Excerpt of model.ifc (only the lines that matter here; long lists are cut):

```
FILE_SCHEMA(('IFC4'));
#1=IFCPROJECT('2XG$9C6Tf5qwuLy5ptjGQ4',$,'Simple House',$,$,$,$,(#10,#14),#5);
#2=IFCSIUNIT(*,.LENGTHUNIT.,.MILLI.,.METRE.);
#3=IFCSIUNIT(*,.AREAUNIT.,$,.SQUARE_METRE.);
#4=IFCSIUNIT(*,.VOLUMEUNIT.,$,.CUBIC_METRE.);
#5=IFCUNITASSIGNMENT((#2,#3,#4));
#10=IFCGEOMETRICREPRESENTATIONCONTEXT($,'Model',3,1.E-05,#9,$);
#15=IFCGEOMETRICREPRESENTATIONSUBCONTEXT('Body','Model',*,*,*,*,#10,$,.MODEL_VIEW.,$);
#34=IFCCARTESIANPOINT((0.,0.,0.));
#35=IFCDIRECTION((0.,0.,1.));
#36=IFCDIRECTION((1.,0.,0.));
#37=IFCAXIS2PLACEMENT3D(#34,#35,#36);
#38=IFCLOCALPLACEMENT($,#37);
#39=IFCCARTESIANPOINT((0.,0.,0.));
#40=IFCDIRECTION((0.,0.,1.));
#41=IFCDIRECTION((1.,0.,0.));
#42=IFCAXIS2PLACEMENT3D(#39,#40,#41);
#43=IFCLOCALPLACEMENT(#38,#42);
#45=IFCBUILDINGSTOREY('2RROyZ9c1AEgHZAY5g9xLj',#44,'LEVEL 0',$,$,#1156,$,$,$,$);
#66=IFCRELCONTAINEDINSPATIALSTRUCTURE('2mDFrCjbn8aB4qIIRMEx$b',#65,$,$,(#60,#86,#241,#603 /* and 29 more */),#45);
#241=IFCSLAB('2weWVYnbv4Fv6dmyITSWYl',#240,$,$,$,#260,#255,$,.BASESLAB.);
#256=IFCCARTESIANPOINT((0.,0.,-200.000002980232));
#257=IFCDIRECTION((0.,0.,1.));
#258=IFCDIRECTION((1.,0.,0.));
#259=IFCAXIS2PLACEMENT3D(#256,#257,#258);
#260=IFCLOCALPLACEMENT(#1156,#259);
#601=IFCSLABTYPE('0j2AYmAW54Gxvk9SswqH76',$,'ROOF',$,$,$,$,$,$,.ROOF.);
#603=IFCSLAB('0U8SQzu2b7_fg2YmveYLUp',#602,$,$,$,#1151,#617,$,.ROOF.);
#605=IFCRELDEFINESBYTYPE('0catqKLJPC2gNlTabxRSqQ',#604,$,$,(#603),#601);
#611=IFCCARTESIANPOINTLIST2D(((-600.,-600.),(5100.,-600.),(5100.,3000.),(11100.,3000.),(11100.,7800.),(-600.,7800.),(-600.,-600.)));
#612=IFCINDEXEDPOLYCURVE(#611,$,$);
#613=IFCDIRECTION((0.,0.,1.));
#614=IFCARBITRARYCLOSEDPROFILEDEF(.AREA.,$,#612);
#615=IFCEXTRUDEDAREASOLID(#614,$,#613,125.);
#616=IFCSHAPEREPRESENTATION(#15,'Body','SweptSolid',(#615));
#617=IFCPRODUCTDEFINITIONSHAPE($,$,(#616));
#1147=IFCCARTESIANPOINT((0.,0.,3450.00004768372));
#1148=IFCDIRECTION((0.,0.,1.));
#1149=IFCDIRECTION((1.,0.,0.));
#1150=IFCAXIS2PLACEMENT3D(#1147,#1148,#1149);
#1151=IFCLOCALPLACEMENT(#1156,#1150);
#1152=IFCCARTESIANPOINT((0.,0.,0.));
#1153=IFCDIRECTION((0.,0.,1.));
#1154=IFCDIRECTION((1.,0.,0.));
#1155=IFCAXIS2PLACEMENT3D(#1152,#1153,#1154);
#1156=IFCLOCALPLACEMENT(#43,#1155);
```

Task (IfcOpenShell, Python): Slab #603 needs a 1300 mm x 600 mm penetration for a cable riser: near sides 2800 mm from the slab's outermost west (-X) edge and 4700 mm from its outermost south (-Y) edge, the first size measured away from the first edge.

```python
import numpy as np
import ifcopenshell
import ifcopenshell.api.feature
import ifcopenshell.api.geometry
import ifcopenshell.api.root
import ifcopenshell.geom
import ifcopenshell.util.placement
import ifcopenshell.util.representation
import ifcopenshell.util.shape
import ifcopenshell.util.unit

model = ifcopenshell.open("model.ifc")
unit_scale = ifcopenshell.util.unit.calculate_unit_scale(model)
settings = ifcopenshell.geom.settings()


def volume(element):
    """Net volume in cubic metres, openings subtracted."""
    shape = ifcopenshell.geom.create_shape(settings, element)
    return ifcopenshell.util.shape.get_volume(shape.geometry)


slab = model.by_guid("0U8SQzu2b7_fg2YmveYLUp")
before = volume(slab)

# Extent in the slab's own axes, in metres. The edges named are its -X and -Y sides.
slab_shape = ifcopenshell.geom.create_shape(settings, slab)
vertices = ifcopenshell.util.shape.get_vertices(slab_shape.geometry)
x_min, y_min, bottom = vertices.min(axis=0)
top = vertices[:, 2].max()

opening = ifcopenshell.api.root.create_entity(model, ifc_class="IfcOpeningElement", name="Cable riser opening", predefined_type="OPENING")
context = ifcopenshell.util.representation.get_context(model, "Model", "Body", "MODEL_VIEW")
width, depth = 1.3, 0.6
outline = [(0.0, 0.0), (width, 0.0), (width, depth), (0.0, depth), (0.0, 0.0)]
# Overshoot both faces by 50 mm so the cut is clean.
shape = ifcopenshell.api.geometry.add_slab_representation(
    model, context=context, depth=top - bottom + 0.1, polyline=outline
)
ifcopenshell.api.geometry.assign_representation(model, product=opening, representation=shape)

matrix = ifcopenshell.util.placement.get_local_placement(slab.ObjectPlacement)
matrix[:, 3] = matrix @ np.append(np.array([x_min + 2.8, y_min + 4.7, bottom - 0.05]) / unit_scale, 1.0)
ifcopenshell.api.geometry.edit_object_placement(model, product=opening, matrix=matrix, is_si=False)
ifcopenshell.api.feature.add_feature(model, feature=opening, element=slab)

after = volume(slab)

print(f"slab volume {before:.3f} -> {after:.3f} m3")

model.write("model_edited.ifc")
```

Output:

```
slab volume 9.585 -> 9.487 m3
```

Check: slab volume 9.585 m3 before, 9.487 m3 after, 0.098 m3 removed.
